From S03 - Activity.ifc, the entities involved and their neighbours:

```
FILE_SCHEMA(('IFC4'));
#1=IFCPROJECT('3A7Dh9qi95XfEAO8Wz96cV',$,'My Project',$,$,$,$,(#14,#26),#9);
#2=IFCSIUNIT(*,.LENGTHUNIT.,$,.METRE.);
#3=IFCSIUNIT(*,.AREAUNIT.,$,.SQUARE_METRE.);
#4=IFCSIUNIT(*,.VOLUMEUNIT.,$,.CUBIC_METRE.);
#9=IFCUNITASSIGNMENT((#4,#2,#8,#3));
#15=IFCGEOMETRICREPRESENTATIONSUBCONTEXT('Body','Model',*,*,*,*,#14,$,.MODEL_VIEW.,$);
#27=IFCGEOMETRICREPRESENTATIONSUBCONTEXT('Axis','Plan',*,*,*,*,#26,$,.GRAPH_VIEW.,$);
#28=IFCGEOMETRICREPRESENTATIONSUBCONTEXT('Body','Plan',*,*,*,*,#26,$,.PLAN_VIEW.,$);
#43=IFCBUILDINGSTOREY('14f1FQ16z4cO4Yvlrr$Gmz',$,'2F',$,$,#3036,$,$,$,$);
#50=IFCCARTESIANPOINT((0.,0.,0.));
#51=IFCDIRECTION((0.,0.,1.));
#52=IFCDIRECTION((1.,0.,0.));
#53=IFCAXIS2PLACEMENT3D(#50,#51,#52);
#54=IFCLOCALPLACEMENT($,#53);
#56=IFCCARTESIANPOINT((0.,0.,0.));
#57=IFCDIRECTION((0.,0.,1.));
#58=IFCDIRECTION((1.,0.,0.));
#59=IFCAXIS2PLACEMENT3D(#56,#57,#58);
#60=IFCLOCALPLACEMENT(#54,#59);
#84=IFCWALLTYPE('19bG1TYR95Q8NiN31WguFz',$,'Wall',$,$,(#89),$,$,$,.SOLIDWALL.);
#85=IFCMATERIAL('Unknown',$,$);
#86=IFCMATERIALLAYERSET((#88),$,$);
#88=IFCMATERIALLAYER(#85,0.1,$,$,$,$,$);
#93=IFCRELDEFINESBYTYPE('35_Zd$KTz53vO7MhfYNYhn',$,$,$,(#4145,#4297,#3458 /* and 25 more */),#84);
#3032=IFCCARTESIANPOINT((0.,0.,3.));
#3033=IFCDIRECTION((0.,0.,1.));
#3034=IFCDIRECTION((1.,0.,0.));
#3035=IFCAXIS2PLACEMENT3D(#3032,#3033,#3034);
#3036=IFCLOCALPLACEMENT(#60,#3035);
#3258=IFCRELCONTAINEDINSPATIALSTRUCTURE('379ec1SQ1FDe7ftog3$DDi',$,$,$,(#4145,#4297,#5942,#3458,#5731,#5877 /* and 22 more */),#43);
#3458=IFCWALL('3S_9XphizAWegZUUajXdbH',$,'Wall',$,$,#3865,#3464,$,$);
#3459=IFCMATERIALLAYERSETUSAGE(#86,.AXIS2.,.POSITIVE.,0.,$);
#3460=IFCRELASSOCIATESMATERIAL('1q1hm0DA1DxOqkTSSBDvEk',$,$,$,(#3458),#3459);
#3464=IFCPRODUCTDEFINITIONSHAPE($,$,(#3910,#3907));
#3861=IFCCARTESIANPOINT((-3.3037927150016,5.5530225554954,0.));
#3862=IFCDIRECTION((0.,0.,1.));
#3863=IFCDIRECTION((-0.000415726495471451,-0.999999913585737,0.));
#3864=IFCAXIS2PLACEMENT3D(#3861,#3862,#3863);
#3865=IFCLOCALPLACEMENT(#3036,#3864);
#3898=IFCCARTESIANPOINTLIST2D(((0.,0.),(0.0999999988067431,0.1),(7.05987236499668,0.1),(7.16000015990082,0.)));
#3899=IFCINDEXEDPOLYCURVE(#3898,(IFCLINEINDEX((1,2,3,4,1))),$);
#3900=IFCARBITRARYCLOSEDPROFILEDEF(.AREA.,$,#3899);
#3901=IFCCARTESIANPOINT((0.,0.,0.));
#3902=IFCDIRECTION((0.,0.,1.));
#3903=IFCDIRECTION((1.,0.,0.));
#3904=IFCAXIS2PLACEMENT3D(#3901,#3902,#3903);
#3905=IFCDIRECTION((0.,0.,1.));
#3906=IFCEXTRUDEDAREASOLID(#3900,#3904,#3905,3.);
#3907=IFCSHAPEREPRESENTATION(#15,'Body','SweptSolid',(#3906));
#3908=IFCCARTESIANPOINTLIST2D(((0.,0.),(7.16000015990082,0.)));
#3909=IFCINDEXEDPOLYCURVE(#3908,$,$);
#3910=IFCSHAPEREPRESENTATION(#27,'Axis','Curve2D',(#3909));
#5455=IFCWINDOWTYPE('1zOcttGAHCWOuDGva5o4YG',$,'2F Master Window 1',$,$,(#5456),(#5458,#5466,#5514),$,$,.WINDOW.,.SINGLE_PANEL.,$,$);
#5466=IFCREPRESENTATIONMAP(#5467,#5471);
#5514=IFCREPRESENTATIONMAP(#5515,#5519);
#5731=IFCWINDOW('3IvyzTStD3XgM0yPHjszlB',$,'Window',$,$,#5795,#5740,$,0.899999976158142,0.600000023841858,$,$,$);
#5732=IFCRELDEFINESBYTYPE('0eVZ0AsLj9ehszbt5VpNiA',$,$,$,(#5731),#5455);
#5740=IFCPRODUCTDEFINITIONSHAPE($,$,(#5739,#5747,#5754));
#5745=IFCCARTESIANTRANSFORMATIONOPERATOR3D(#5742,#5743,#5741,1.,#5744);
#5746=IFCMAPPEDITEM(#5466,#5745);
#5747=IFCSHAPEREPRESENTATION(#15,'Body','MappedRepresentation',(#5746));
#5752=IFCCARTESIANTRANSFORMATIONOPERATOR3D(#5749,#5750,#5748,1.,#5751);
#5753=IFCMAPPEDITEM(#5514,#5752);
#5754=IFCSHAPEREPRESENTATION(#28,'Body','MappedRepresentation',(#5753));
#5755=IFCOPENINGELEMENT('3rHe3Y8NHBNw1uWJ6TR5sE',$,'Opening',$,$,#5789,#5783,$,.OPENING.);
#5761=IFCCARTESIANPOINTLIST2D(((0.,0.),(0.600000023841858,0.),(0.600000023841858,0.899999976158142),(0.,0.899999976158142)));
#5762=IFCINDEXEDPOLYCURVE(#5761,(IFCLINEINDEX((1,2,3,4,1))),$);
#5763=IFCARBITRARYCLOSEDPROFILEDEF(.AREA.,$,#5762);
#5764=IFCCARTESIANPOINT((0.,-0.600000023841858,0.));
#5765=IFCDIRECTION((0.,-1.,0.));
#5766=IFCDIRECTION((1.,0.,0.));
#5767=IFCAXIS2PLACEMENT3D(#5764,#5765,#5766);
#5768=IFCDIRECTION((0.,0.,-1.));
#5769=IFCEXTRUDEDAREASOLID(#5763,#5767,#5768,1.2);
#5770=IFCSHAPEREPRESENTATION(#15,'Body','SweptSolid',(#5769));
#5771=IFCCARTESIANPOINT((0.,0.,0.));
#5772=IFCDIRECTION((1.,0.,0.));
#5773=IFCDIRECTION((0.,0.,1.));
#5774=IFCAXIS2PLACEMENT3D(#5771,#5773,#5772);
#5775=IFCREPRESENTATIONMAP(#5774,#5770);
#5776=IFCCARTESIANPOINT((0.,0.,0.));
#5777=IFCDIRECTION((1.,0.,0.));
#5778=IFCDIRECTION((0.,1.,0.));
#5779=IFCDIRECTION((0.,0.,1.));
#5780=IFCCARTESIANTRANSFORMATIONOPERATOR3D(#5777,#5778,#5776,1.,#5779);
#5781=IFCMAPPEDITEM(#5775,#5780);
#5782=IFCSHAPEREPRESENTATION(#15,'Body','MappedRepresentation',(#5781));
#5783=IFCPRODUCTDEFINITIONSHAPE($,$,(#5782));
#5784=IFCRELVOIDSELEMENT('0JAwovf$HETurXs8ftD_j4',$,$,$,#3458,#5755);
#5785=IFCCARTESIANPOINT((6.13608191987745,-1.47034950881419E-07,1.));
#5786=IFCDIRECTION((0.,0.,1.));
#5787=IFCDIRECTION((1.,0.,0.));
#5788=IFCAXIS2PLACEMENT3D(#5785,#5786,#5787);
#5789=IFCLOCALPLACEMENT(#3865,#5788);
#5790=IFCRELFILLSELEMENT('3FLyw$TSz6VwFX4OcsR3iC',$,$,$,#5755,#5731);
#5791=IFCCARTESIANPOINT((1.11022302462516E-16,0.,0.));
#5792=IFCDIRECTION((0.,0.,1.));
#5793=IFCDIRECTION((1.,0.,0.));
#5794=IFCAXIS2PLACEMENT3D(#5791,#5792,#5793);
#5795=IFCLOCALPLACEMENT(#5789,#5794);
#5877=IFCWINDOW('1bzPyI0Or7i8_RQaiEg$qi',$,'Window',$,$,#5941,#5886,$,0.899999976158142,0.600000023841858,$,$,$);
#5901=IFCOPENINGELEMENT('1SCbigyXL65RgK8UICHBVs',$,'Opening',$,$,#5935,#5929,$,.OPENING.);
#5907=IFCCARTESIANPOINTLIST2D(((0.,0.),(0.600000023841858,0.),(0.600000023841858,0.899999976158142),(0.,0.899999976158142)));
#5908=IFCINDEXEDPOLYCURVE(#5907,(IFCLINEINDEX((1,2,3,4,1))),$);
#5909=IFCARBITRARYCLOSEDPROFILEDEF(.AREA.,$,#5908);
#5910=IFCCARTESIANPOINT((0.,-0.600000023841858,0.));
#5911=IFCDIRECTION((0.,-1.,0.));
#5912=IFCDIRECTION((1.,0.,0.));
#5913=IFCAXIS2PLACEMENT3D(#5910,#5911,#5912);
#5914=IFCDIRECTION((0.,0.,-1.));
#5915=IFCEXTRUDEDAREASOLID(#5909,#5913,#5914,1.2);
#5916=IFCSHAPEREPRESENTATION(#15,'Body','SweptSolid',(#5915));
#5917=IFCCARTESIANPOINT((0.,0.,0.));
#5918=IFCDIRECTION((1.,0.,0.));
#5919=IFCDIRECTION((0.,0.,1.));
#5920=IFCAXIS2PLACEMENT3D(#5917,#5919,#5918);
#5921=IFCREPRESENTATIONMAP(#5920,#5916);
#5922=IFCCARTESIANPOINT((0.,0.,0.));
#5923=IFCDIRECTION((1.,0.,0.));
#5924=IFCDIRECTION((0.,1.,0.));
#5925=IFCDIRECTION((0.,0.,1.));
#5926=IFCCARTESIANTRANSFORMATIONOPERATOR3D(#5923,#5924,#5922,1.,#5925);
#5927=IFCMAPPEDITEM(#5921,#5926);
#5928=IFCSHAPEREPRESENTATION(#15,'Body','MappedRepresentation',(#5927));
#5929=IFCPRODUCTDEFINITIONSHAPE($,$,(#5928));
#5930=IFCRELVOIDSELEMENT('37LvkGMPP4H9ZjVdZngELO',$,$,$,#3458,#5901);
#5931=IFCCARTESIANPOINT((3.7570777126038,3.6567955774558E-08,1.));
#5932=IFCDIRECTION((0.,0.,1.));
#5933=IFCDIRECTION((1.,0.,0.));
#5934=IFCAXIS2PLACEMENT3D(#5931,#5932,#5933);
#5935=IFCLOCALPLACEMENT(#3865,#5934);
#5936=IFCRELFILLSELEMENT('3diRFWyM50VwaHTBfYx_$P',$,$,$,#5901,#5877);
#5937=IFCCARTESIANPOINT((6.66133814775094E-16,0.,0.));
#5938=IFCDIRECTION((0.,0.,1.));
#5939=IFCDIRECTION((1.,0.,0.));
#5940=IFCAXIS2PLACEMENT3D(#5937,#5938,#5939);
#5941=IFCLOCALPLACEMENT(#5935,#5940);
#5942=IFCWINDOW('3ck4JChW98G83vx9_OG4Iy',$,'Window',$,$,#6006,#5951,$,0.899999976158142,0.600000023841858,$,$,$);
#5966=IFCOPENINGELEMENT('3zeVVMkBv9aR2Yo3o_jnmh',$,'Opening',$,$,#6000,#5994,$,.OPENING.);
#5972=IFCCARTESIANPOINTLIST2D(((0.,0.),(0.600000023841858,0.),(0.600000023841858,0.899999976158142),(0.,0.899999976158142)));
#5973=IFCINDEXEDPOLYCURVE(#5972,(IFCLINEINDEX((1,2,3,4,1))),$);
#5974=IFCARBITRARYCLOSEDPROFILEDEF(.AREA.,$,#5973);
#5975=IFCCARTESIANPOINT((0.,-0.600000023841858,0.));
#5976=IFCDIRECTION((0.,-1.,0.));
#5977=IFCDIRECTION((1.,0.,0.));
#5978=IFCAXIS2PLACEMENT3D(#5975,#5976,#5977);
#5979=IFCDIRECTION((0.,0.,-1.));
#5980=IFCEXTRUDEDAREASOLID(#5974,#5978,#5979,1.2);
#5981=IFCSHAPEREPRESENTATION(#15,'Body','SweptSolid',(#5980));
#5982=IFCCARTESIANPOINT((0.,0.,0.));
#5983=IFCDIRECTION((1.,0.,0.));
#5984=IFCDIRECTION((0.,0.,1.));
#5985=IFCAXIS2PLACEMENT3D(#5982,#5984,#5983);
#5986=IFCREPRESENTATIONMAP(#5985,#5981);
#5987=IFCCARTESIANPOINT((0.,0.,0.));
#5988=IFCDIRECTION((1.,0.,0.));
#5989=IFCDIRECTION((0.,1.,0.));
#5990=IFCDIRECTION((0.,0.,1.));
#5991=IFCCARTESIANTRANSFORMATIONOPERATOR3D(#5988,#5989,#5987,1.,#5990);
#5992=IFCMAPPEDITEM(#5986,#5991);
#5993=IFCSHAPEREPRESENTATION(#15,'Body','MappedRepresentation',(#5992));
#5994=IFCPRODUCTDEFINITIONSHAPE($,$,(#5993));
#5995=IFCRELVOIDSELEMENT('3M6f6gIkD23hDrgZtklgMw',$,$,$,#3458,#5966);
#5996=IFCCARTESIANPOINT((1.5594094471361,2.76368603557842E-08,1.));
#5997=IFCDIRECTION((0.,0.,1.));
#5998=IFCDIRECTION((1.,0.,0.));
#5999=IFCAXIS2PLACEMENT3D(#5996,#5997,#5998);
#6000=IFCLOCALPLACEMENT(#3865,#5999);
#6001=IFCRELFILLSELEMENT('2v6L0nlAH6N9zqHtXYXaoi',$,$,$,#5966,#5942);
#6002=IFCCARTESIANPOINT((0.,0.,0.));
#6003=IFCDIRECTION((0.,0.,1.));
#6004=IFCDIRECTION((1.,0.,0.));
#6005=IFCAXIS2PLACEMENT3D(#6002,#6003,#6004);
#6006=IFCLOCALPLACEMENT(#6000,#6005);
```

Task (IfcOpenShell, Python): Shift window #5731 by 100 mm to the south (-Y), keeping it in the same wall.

```python
import ifcopenshell
import ifcopenshell.api.geometry
import ifcopenshell.util.placement
import ifcopenshell.util.unit

model = ifcopenshell.open("S03 - Activity.ifc")
unit_scale = ifcopenshell.util.unit.calculate_unit_scale(model)

window = model.by_guid("3IvyzTStD3XgM0yPHjszlB")
opening = window.FillsVoids[0].RelatingOpeningElement
wall = opening.VoidsElements[0].RelatingBuildingElement

wall_matrix = ifcopenshell.util.placement.get_local_placement(wall.ObjectPlacement)
shift = wall_matrix[:3, 0] * 0.1 / unit_scale
before = ifcopenshell.util.placement.get_local_placement(window.ObjectPlacement)[:3, 3].copy()

# The window is placed relative to its opening, so it follows when the opening moves.
matrix = ifcopenshell.util.placement.get_local_placement(opening.ObjectPlacement)
matrix[:3, 3] += shift
ifcopenshell.api.geometry.edit_object_placement(
    model, product=opening, matrix=matrix, is_si=False, should_transform_children=True
)

after = ifcopenshell.util.placement.get_local_placement(window.ObjectPlacement)[:3, 3]
print("window moved by", (after - before).round(3) + 0.0)

model.write("S03 - Activity_v2.ifc")
```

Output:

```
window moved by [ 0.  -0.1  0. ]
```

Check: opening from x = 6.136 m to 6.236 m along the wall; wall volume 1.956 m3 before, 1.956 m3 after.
